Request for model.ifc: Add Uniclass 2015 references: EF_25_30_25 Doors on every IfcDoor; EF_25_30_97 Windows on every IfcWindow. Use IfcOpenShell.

First a look at what the model holds.

```python
import ifcopenshell

model = ifcopenshell.open("model.ifc")
print(model.schema)
print("classifications:", [c.Name for c in model.by_type("IfcClassification")])
for ifc_class in ("IfcDoor", "IfcRoof", "IfcStair", "IfcWall", "IfcWindow"):
    print(ifc_class, len(model.by_type(ifc_class)))
```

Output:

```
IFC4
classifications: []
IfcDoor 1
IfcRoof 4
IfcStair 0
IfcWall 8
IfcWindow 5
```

```python
import ifcopenshell
import ifcopenshell.api.classification

model = ifcopenshell.open("model.ifc")

system = ifcopenshell.api.classification.add_classification(model, classification="Uniclass 2015")

codes = {
    "IfcDoor": ("EF_25_30_25", "Doors"),
    "IfcWindow": ("EF_25_30_97", "Windows"),
}
for ifc_class, (code, name) in codes.items():
    products = model.by_type(ifc_class)
    ifcopenshell.api.classification.add_reference(
        model, products=products, classification=system, identification=code, name=name
    )
    print(code, len(products))

model.write("model_rev.ifc")
```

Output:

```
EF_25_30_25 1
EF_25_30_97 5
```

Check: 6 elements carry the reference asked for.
